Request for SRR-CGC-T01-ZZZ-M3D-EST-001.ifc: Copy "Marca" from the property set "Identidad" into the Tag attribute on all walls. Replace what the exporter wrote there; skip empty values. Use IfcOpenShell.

First a look at what the model holds.

```python
import ifcopenshell
import ifcopenshell.util.element

model = ifcopenshell.open("SRR-CGC-T01-ZZZ-M3D-EST-001.ifc")
print(model.schema)
walls = model.by_type("IfcWall")
print(len(walls), "walls")
for e in walls[:8]:
    source = ifcopenshell.util.element.get_pset(e, "Identidad", "Marca")
    target = e.Tag
    print(e.id(), repr(source), repr(target), sep=" | ")
```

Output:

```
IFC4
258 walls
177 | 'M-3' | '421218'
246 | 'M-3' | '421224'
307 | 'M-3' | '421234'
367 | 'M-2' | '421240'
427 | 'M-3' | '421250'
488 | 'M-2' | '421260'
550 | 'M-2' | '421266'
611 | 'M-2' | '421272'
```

```python
import ifcopenshell
import ifcopenshell.util.element

model = ifcopenshell.open("SRR-CGC-T01-ZZZ-M3D-EST-001.ifc")

count = 0
for e in model.by_type("IfcWall"):
    value = ifcopenshell.util.element.get_pset(e, "Identidad", "Marca")
    current = e.Tag
    if not value or not value.strip() or current == value:
        continue
    e.Tag = value
    count += 1

print(count, "walls updated")

model.write("SRR-CGC-T01-ZZZ-M3D-EST-001_edited.ifc")
```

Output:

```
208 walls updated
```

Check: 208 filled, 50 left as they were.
